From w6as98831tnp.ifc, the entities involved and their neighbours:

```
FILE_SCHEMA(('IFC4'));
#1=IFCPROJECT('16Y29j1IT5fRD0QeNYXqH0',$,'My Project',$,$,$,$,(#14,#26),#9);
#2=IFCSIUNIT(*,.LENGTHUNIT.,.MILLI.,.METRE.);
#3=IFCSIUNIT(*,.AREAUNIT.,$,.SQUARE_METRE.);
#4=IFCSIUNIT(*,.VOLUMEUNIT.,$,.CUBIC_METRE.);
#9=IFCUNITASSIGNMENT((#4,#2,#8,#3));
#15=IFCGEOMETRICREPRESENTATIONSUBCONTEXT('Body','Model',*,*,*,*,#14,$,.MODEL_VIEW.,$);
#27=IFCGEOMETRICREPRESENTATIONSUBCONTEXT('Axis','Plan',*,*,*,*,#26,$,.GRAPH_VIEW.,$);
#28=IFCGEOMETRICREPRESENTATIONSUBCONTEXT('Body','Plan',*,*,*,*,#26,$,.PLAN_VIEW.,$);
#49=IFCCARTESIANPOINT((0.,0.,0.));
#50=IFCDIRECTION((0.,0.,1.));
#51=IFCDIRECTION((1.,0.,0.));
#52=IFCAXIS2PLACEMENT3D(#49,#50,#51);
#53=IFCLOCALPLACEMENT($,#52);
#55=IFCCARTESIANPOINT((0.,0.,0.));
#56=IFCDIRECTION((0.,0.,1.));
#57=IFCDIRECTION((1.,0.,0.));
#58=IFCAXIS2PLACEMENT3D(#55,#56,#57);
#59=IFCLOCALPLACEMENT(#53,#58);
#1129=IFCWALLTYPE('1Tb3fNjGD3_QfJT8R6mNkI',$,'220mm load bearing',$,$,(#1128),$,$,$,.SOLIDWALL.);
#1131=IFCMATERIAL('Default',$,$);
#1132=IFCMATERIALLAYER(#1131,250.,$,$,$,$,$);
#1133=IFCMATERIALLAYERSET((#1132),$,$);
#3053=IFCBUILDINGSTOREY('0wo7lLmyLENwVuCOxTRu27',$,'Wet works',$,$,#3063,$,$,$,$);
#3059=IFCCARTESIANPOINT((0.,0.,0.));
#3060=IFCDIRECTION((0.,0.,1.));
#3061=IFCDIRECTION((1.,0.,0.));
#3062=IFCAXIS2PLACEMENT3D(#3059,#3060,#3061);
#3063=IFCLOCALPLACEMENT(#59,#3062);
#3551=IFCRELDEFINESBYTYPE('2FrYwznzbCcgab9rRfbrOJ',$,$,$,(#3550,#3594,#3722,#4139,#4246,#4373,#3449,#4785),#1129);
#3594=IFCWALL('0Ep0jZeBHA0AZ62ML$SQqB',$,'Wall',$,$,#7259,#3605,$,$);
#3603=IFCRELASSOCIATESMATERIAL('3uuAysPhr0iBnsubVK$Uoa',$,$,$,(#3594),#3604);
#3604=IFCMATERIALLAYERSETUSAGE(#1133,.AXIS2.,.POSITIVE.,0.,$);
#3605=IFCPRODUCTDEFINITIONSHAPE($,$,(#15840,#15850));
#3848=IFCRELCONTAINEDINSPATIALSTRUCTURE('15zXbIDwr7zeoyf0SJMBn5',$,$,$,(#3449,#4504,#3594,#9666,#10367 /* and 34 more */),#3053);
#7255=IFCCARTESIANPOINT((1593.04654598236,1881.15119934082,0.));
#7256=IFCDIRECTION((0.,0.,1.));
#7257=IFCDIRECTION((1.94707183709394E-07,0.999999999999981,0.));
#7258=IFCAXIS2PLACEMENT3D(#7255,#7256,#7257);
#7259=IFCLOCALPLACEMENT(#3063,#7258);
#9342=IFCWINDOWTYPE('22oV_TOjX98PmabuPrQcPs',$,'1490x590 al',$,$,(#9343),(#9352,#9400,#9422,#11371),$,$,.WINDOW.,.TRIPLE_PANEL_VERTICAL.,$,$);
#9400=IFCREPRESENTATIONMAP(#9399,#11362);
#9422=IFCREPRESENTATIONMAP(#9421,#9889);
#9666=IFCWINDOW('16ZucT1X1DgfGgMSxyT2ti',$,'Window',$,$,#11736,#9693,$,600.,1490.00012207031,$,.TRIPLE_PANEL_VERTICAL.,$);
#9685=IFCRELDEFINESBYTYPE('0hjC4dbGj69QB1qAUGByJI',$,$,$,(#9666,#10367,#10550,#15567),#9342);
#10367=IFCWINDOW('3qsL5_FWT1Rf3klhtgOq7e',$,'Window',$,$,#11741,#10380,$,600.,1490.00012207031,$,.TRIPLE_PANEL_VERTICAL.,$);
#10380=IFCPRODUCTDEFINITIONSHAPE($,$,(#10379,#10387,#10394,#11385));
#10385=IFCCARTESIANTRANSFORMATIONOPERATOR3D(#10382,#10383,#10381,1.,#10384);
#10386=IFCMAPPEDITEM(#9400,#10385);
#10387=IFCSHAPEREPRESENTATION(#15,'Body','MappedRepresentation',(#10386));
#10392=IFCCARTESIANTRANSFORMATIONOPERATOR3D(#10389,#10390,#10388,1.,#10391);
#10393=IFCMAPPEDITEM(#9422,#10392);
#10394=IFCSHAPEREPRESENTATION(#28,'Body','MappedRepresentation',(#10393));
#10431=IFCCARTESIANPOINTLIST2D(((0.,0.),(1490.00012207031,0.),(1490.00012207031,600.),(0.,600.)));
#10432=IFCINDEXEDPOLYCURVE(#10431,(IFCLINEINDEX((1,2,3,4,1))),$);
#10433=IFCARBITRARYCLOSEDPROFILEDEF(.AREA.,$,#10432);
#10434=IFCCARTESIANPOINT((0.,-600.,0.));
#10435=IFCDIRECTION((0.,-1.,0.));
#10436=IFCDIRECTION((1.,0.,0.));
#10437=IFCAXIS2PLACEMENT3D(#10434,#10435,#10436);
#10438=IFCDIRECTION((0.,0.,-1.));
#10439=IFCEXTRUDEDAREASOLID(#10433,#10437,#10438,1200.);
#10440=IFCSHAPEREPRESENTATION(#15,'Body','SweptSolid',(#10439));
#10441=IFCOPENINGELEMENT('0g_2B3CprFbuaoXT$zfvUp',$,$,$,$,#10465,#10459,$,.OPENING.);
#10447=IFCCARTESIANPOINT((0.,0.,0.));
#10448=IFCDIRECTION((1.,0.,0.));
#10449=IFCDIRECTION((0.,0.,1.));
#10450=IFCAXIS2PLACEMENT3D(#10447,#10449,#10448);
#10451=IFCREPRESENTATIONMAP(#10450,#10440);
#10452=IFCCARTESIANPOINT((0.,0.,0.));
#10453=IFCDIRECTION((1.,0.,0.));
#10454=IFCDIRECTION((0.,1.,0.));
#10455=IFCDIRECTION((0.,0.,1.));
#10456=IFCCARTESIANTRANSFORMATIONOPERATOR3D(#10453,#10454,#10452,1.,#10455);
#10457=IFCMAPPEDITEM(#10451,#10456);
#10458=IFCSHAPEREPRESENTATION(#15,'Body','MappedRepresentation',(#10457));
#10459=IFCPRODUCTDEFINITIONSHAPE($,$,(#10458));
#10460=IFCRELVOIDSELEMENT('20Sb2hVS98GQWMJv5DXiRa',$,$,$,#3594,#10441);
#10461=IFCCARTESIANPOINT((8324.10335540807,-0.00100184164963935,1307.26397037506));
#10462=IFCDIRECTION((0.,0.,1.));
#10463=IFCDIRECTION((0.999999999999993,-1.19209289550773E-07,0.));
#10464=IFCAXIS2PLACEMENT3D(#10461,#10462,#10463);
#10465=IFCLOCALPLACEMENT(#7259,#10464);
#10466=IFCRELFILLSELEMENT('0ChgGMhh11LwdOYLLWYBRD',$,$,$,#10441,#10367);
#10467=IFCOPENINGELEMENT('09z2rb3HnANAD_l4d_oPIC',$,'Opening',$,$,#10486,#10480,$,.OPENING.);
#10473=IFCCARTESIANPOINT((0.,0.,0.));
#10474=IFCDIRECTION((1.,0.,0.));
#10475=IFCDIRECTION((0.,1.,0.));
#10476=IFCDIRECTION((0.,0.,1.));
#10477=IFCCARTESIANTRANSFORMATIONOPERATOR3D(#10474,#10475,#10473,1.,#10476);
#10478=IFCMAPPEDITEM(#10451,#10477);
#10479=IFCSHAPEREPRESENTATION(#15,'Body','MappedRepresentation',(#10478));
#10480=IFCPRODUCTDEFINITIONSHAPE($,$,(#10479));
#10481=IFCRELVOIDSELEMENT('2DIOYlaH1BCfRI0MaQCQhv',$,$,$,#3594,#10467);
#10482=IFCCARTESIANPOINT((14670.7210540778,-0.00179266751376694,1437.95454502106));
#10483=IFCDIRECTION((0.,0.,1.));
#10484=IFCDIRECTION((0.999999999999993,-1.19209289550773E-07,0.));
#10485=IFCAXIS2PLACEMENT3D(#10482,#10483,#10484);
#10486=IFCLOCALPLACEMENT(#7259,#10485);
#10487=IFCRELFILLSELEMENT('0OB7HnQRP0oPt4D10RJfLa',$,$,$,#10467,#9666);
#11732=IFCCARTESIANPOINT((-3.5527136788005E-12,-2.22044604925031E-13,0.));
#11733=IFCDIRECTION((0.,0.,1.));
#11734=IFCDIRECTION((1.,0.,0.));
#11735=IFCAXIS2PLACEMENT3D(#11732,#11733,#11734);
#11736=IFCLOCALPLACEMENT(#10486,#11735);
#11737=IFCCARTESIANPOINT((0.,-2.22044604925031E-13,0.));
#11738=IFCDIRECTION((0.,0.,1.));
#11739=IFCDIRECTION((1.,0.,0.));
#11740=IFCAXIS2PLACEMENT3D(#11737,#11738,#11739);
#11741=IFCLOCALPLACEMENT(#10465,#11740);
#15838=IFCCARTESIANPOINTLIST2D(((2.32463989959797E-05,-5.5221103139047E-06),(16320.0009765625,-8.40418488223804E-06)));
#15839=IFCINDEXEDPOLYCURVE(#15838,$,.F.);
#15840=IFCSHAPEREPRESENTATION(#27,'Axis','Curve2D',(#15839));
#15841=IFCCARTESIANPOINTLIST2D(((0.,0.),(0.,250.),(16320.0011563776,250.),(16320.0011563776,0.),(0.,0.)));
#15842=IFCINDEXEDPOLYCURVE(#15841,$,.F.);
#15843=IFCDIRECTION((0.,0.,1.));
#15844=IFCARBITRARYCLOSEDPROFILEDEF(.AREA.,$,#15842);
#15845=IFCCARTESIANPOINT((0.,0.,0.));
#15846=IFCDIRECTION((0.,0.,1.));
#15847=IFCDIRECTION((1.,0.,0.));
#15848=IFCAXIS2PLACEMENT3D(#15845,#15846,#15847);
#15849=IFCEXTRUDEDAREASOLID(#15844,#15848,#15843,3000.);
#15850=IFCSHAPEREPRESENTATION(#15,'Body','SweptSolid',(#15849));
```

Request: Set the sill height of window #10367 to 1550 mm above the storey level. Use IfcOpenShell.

```python
import numpy as np
import ifcopenshell
import ifcopenshell.api.geometry
import ifcopenshell.geom
import ifcopenshell.util.element
import ifcopenshell.util.placement
import ifcopenshell.util.shape
import ifcopenshell.util.unit

model = ifcopenshell.open("w6as98831tnp.ifc")
unit_scale = ifcopenshell.util.unit.calculate_unit_scale(model)

window = model.by_guid("3qsL5_FWT1Rf3klhtgOq7e")
opening = window.FillsVoids[0].RelatingOpeningElement
storey = ifcopenshell.util.element.get_container(window, ifc_class="IfcBuildingStorey")
level = ifcopenshell.util.placement.get_local_placement(storey.ObjectPlacement)[2, 3]

# The opening's origin need not be at the sill, so measure its lowest point.
shape = ifcopenshell.geom.create_shape(ifcopenshell.geom.settings(), opening)
bottom = ifcopenshell.util.shape.get_shape_bottom_elevation(shape, shape.geometry) / unit_scale
dz = level + 1.55 / unit_scale - bottom

shift = np.array([0.0, 0.0, dz])
# The window is placed relative to its opening, so it follows when the opening moves.
matrix = ifcopenshell.util.placement.get_local_placement(opening.ObjectPlacement)
matrix[:3, 3] += shift
ifcopenshell.api.geometry.edit_object_placement(
    model, product=opening, matrix=matrix, is_si=False, should_transform_children=True
)

print(f"moved by {dz * unit_scale:+.3f} m")

model.write("w6as98831tnp_updated.ifc")
```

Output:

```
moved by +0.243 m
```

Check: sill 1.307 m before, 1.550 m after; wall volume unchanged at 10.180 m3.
